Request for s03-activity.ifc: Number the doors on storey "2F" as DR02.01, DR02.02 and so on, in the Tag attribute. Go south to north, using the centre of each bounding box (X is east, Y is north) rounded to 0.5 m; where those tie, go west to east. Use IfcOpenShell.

First a look at what the model holds.

```python
import ifcopenshell
import ifcopenshell.util.element
import ifcopenshell.util.placement

model = ifcopenshell.open("s03-activity.ifc")
print(model.schema)
storey = next(s for s in model.by_type("IfcBuildingStorey") if s.Name == "2F")
doors = [e for e in ifcopenshell.util.element.get_decomposition(storey) if e.is_a("IfcDoor")]
for e in sorted(doors, key=lambda e: e.id()):
    origin = ifcopenshell.util.placement.get_local_placement(e.ObjectPlacement)[:3, 3]
    print(e.id(), e.Tag, e.Name, origin.round(2) + 0.0, sep=" | ")
```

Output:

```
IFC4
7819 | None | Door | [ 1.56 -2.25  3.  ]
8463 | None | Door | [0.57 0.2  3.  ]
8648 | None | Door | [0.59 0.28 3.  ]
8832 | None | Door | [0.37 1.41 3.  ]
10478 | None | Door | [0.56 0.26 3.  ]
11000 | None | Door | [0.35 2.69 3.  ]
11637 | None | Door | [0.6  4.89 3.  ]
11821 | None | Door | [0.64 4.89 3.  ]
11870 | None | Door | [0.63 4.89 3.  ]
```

```python
import ifcopenshell
import ifcopenshell.geom
import ifcopenshell.util.element
import ifcopenshell.util.shape

model = ifcopenshell.open("s03-activity.ifc")
settings = ifcopenshell.geom.settings()
settings.set("use-world-coords", True)


def centre(element):
    shape = ifcopenshell.geom.create_shape(settings, element)
    return ifcopenshell.util.shape.get_bbox_centroid(shape.geometry)


storey = next(s for s in model.by_type("IfcBuildingStorey") if s.Name == "2F")
doors = [e for e in ifcopenshell.util.element.get_decomposition(storey) if e.is_a("IfcDoor")]

# Insertion points can sit at a corner or the storey origin, so sort by the geometry (in metres).
centres = {e: centre(e) for e in doors}
doors.sort(key=lambda e: (round(centres[e][1] / 0.5), centres[e][0]))

for i, e in enumerate(doors, start=1):
    number = f"DR02.{i:02d}"
    e.Tag = number
    print(e.id(), number)

model.write("s03-activity_rev.ifc")
```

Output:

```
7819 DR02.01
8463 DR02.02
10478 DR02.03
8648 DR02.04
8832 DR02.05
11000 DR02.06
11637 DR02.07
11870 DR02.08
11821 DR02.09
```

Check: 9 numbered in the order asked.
